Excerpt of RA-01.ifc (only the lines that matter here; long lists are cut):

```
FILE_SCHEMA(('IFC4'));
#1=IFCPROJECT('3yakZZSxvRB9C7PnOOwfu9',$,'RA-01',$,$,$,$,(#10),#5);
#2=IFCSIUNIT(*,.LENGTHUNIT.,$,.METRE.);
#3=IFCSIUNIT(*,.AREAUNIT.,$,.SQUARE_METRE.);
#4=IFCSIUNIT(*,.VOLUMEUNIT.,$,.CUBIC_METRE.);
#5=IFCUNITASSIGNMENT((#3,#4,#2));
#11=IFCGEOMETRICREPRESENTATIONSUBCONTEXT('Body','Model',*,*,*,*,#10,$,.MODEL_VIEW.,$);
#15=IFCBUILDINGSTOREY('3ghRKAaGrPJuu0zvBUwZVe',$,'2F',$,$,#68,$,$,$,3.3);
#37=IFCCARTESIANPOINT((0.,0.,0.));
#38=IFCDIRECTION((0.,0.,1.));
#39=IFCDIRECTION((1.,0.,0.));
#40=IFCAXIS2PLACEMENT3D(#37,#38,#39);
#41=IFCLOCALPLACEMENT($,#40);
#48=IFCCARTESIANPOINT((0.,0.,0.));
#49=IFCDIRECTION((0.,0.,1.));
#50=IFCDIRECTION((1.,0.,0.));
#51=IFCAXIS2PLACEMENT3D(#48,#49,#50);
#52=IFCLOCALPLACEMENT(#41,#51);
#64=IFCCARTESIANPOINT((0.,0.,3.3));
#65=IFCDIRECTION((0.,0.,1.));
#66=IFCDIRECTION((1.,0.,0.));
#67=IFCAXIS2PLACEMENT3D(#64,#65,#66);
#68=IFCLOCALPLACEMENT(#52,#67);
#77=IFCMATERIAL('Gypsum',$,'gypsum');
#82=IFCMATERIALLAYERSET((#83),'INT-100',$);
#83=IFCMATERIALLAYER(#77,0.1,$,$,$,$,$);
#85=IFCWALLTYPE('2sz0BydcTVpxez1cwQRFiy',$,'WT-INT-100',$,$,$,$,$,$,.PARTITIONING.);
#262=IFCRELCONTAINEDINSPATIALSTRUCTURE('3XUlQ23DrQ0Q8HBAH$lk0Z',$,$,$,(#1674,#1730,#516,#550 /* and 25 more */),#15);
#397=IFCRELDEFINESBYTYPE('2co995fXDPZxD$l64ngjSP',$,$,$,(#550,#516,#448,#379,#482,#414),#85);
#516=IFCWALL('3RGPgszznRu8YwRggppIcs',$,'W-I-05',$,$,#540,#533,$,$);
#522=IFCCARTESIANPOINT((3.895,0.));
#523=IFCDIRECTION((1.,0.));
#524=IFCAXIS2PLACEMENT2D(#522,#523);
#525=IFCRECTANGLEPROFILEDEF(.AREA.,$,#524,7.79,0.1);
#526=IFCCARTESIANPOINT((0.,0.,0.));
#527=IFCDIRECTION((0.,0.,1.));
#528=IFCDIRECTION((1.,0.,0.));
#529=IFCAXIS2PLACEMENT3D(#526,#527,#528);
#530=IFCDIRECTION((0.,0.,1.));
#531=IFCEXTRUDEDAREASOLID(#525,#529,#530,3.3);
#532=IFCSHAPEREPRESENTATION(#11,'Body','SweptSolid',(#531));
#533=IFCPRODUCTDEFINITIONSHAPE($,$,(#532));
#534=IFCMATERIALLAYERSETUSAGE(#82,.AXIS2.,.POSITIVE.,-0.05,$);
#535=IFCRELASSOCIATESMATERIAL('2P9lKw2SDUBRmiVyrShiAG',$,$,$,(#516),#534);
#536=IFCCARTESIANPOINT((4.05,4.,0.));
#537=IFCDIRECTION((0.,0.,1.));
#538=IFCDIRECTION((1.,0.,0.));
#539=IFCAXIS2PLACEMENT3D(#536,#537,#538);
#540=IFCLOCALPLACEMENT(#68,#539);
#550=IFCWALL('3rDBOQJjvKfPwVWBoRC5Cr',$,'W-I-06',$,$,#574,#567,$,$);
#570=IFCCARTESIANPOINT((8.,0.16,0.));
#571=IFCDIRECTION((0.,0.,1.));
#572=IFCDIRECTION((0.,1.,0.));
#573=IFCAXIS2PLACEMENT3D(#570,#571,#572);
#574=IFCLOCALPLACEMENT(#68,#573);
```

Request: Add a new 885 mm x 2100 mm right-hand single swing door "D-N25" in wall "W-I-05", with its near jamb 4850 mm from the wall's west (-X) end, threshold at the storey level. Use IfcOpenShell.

```python
import numpy as np
import ifcopenshell
import ifcopenshell.api.feature
import ifcopenshell.api.geometry
import ifcopenshell.api.root
import ifcopenshell.api.spatial
import ifcopenshell.geom
import ifcopenshell.util.element
import ifcopenshell.util.placement
import ifcopenshell.util.representation
import ifcopenshell.util.shape
import ifcopenshell.util.unit

model = ifcopenshell.open("RA-01.ifc")
unit_scale = ifcopenshell.util.unit.calculate_unit_scale(model)
settings = ifcopenshell.geom.settings()


def volume(element):
    """Net volume in cubic metres, openings subtracted."""
    shape = ifcopenshell.geom.create_shape(settings, element)
    return ifcopenshell.util.shape.get_volume(shape.geometry)


wall = model.by_guid("3RGPgszznRu8YwRggppIcs")
storey = ifcopenshell.util.element.get_container(wall, ifc_class="IfcBuildingStorey")
context = ifcopenshell.util.representation.get_context(model, "Model", "Body", "MODEL_VIEW")
before = volume(wall)

width, height, from_end, sill = 0.885, 2.1, 4.85, 0.0  # metres

# The wall runs along its own X axis, and the end named is its -X end.
wall_shape = ifcopenshell.geom.create_shape(settings, wall)
x, y, z = ifcopenshell.util.shape.get_vertices(wall_shape.geometry).T
start = x.min() + from_end
face, thickness = float(y.min()), float(y.max() - y.min())
wall_matrix = ifcopenshell.util.placement.get_local_placement(wall.ObjectPlacement)
level = ifcopenshell.util.placement.get_local_placement(storey.ObjectPlacement)[2, 3]


def in_wall(x, y):
    """Placement at x, y metres in the wall's axes, at sill height."""
    matrix = wall_matrix.copy()
    matrix[:, 3] = wall_matrix @ np.array([x / unit_scale, y / unit_scale, 0.0, 1.0])
    matrix[2, 3] = level + sill / unit_scale
    return matrix


# Opening: a box that overshoots both wall faces by 50 mm.
opening = ifcopenshell.api.root.create_entity(model, ifc_class="IfcOpeningElement", predefined_type="OPENING")
box = ifcopenshell.api.geometry.add_wall_representation(
    model, context=context, length=width, height=height, thickness=thickness + 0.1
)
ifcopenshell.api.geometry.assign_representation(model, product=opening, representation=box)
ifcopenshell.api.geometry.edit_object_placement(model, product=opening, matrix=in_wall(start, face - 0.05), is_si=False)
ifcopenshell.api.feature.add_feature(model, feature=opening, element=wall)

door = ifcopenshell.api.root.create_entity(model, ifc_class="IfcDoor", name="D-N25", predefined_type="DOOR")
door.OverallWidth, door.OverallHeight = width / unit_scale, height / unit_scale
door.OperationType = "SINGLE_SWING_RIGHT"
body = ifcopenshell.api.geometry.add_door_representation(
    model,
    context=context,
    overall_width=door.OverallWidth,
    overall_height=door.OverallHeight,
    operation_type="SINGLE_SWING_RIGHT",
    lining_properties={"LiningDepth": thickness / unit_scale, "ThresholdDepth": thickness / unit_scale},
)
ifcopenshell.api.geometry.assign_representation(model, product=door, representation=body)
ifcopenshell.api.spatial.assign_container(model, products=[door], relating_structure=storey)
ifcopenshell.api.feature.add_filling(model, opening=opening, element=door)

# The lining spans the wall, so the door starts at the wall face.
ifcopenshell.api.geometry.edit_object_placement(model, product=door, matrix=in_wall(start, face), is_si=False)

after = volume(wall)

print(f"wall volume {before:.3f} -> {after:.3f} m3")

model.write("RA-01_v2.ifc")
```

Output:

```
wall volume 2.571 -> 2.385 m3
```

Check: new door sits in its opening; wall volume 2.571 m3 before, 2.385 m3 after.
